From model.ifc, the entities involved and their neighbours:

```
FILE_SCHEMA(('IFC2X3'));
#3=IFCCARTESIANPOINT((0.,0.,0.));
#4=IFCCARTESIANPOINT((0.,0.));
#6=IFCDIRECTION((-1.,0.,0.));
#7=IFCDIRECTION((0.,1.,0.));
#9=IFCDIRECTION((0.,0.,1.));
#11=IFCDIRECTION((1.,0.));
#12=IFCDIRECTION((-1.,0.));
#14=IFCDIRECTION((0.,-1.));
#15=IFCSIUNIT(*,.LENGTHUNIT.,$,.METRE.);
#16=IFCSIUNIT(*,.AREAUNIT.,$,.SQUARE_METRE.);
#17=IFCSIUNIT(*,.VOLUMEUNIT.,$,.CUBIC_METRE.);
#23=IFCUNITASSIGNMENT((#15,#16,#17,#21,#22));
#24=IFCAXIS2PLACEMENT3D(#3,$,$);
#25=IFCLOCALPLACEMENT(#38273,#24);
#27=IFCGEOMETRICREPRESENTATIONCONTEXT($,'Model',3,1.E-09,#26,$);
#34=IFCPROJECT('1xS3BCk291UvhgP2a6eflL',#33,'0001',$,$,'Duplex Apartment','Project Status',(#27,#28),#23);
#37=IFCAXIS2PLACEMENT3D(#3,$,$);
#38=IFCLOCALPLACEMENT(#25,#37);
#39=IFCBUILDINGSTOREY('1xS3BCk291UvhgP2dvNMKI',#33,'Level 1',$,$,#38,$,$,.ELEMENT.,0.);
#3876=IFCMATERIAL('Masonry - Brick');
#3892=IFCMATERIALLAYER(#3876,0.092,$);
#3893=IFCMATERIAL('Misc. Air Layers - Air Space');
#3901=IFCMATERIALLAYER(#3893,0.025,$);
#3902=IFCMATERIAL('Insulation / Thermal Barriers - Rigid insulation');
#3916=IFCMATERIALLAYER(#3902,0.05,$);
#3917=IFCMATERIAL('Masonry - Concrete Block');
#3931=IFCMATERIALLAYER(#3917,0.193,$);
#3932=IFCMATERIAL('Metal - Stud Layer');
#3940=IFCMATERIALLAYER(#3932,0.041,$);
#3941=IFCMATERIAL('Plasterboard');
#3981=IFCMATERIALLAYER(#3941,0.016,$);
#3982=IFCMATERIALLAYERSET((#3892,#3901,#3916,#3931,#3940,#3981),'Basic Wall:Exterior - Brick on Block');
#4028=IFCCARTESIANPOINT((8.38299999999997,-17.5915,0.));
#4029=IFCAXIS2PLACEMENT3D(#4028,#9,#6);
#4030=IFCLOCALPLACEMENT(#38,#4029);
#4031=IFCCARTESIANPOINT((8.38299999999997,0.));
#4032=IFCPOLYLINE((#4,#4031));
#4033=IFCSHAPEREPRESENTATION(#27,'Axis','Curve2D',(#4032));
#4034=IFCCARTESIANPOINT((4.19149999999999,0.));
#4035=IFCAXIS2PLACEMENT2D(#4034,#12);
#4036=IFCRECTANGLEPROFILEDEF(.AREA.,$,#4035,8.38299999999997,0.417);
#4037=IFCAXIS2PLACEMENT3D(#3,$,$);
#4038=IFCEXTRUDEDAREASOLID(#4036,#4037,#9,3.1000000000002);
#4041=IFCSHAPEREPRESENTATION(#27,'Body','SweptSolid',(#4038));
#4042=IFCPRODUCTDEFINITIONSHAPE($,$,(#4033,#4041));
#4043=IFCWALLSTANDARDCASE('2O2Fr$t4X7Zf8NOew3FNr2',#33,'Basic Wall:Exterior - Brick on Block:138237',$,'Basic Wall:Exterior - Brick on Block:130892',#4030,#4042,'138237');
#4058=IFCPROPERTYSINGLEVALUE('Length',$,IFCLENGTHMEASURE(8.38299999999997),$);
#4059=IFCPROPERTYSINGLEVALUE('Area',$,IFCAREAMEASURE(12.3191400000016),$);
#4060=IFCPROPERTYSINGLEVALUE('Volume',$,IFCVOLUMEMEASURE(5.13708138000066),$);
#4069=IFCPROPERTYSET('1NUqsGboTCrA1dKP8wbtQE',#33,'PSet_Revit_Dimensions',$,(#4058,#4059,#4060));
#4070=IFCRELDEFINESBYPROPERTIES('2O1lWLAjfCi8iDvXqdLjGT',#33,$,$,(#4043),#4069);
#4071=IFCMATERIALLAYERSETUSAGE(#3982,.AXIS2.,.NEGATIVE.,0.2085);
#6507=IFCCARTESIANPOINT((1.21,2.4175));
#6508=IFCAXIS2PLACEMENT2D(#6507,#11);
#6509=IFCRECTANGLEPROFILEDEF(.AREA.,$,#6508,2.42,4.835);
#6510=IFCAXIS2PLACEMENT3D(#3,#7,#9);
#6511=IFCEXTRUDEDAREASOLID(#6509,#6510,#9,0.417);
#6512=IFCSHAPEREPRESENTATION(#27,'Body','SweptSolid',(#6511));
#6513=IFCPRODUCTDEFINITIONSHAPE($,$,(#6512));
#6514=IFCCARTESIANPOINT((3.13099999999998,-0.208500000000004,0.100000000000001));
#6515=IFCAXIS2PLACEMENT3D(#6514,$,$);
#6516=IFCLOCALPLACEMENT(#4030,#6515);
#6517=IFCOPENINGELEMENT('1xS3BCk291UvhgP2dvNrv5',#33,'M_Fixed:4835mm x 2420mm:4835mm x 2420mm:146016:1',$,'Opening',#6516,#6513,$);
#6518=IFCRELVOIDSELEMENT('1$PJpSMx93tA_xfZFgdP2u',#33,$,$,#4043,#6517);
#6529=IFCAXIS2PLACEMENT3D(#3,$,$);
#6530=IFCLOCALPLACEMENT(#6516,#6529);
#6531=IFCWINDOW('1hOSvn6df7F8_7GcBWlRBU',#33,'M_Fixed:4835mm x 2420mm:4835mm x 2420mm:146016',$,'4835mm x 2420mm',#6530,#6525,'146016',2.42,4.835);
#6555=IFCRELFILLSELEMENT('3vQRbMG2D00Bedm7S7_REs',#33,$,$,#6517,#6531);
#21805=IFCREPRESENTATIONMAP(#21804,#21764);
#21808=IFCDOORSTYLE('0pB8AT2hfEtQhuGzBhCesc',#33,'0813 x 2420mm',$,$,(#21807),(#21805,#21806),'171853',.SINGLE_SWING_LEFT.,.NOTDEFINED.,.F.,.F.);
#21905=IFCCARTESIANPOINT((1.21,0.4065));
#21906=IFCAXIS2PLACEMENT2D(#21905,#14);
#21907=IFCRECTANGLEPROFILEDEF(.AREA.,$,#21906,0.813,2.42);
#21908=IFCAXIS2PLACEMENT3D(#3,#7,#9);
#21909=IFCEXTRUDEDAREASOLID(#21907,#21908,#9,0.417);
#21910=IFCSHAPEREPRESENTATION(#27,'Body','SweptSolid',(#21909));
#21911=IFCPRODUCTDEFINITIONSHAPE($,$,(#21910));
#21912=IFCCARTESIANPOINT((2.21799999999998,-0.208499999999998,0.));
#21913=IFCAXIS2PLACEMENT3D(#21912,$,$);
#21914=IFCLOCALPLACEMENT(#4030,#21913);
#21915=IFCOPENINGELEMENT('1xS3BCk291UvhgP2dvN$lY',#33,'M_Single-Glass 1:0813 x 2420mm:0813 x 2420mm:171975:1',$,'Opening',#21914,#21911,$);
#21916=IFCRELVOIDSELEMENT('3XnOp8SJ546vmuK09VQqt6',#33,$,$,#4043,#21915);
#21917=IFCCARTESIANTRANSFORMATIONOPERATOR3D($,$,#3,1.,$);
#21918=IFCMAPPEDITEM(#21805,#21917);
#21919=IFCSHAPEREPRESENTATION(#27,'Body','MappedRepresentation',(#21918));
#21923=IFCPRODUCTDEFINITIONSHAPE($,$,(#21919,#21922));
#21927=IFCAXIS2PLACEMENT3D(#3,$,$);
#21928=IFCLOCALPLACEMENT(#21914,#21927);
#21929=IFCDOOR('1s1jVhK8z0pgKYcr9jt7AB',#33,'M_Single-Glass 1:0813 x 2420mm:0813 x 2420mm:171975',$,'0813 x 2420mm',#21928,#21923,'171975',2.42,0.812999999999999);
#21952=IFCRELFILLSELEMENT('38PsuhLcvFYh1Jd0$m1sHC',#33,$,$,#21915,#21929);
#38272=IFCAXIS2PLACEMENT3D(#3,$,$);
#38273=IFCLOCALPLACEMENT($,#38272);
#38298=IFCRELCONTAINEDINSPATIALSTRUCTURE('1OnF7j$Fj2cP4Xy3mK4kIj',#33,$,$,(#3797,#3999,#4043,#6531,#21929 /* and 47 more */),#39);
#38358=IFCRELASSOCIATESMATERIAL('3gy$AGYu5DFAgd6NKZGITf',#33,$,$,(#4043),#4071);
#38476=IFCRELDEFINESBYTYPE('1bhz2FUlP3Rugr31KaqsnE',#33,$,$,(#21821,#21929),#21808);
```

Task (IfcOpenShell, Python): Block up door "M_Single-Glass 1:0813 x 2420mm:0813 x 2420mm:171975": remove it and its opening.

```python
import ifcopenshell
import ifcopenshell.api.feature
import ifcopenshell.api.pset
import ifcopenshell.api.root
import ifcopenshell.geom
import ifcopenshell.util.element
import ifcopenshell.util.shape
import ifcopenshell.util.unit

model = ifcopenshell.open("model.ifc")
area_scale = ifcopenshell.util.unit.calculate_unit_scale(model, "AREAUNIT")
volume_scale = ifcopenshell.util.unit.calculate_unit_scale(model, "VOLUMEUNIT")
settings = ifcopenshell.geom.settings()


def volume(element):
    """Net volume in cubic metres, openings subtracted."""
    shape = ifcopenshell.geom.create_shape(settings, element)
    return ifcopenshell.util.shape.get_volume(shape.geometry)


door = model.by_guid("1s1jVhK8z0pgKYcr9jt7AB")
opening = door.FillsVoids[0].RelatingOpeningElement
wall = opening.VoidsElements[0].RelatingBuildingElement
before = volume(wall)

ifcopenshell.api.root.remove_product(model, product=door)
ifcopenshell.api.feature.remove_feature(model, feature=opening)

after = volume(wall)
thickness = 0.417  # wall thickness in metres

# Update the wall's stored quantities.
pset = model.by_id(ifcopenshell.util.element.get_pset(wall, "PSet_Revit_Dimensions", should_inherit=False)["id"])
ifcopenshell.api.pset.edit_pset(model, pset=pset, properties={
    "Area": model.create_entity("IfcAreaMeasure", after / thickness / area_scale),
    "Volume": model.create_entity("IfcVolumeMeasure", after / volume_scale),
})

print(f"wall volume {before:.3f} -> {after:.3f} m3")

model.write("model-out.ifc")
```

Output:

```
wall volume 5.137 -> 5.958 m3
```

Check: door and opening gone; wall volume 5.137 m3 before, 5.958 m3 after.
